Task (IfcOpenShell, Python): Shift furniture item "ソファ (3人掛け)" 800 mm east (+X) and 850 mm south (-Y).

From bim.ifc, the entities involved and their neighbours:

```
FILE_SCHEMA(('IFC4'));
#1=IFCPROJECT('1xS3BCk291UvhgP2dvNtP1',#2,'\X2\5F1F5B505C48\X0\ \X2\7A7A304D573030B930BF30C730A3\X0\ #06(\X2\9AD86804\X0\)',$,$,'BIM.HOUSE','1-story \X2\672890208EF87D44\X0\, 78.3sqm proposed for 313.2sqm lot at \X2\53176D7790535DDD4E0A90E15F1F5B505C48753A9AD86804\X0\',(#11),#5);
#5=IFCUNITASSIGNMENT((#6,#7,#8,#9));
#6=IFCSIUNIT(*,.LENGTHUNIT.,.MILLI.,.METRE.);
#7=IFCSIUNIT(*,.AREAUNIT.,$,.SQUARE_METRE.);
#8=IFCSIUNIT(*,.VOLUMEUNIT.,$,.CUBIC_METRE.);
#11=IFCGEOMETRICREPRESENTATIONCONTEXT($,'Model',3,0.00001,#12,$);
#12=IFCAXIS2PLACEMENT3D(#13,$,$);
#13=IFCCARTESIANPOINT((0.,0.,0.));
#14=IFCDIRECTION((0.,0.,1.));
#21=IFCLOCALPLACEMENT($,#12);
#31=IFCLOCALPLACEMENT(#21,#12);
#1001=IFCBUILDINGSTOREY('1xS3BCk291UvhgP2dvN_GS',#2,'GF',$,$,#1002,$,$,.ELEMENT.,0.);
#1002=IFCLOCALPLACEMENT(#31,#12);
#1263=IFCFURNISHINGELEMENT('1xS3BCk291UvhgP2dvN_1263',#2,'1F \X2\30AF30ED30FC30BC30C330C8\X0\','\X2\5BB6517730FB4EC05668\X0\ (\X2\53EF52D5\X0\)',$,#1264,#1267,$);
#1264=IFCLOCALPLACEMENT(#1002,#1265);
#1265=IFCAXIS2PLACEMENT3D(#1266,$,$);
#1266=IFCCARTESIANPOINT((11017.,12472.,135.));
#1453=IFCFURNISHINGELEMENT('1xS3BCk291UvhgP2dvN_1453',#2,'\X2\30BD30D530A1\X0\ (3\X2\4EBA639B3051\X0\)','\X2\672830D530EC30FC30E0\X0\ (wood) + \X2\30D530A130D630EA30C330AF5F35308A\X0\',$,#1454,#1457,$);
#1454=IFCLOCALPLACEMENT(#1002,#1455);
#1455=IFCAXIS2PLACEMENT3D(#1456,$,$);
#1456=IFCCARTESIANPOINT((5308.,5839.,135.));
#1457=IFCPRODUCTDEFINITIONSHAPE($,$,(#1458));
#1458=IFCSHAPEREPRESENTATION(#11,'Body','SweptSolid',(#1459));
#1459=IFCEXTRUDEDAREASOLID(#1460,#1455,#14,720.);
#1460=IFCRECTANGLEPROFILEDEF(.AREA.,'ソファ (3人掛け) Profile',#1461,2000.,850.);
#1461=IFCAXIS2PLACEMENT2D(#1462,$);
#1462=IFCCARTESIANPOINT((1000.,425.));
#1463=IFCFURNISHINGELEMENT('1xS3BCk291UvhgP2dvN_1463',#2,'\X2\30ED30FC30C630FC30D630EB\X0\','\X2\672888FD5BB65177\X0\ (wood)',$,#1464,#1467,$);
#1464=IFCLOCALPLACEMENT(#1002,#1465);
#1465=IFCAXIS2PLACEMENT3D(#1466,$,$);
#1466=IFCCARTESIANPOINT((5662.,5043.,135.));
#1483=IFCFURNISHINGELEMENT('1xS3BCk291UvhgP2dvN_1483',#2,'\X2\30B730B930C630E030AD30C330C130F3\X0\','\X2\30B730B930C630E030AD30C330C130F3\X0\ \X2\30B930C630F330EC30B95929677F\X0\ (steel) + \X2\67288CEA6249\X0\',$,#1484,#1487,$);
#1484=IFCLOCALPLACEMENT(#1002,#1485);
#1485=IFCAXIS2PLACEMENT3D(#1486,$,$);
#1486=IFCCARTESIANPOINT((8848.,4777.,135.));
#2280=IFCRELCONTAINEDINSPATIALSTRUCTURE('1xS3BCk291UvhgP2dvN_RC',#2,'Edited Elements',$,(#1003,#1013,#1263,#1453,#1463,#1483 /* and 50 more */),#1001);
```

```python
import ifcopenshell
import ifcopenshell.api.geometry
import ifcopenshell.util.placement
import ifcopenshell.util.unit

model = ifcopenshell.open("bim.ifc")
unit_scale = ifcopenshell.util.unit.calculate_unit_scale(model)

item = model.by_guid("1xS3BCk291UvhgP2dvN_1453")
matrix = ifcopenshell.util.placement.get_local_placement(item.ObjectPlacement)
matrix[0, 3] += 0.8 / unit_scale
matrix[1, 3] -= 0.85 / unit_scale
ifcopenshell.api.geometry.edit_object_placement(model, product=item, matrix=matrix, is_si=False)

print(ifcopenshell.util.placement.get_local_placement(item.ObjectPlacement).round(3) + 0.0)

model.write("bim_updated.ifc")
```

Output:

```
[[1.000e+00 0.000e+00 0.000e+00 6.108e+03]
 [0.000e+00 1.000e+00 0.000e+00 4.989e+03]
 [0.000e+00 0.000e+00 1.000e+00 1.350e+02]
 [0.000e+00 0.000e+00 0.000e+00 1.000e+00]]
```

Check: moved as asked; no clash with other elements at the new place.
